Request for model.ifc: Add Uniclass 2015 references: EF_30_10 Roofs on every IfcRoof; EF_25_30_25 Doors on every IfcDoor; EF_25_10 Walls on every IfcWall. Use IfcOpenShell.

First a look at what the model holds.

```python
import ifcopenshell

model = ifcopenshell.open("model.ifc")
print(model.schema)
print("classifications:", [c.Name for c in model.by_type("IfcClassification")])
for ifc_class in ("IfcDoor", "IfcRoof", "IfcStair", "IfcWall", "IfcWindow"):
    print(ifc_class, len(model.by_type(ifc_class)))
```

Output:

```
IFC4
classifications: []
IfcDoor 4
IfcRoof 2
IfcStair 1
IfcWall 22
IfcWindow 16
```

```python
import ifcopenshell
import ifcopenshell.api.classification

model = ifcopenshell.open("model.ifc")

system = ifcopenshell.api.classification.add_classification(model, classification="Uniclass 2015")

codes = {
    "IfcRoof": ("EF_30_10", "Roofs"),
    "IfcDoor": ("EF_25_30_25", "Doors"),
    "IfcWall": ("EF_25_10", "Walls"),
}
for ifc_class, (code, name) in codes.items():
    products = model.by_type(ifc_class)
    ifcopenshell.api.classification.add_reference(
        model, products=products, classification=system, identification=code, name=name
    )
    print(code, len(products))

model.write("model-out.ifc")
```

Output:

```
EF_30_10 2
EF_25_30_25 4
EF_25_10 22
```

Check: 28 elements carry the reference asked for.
